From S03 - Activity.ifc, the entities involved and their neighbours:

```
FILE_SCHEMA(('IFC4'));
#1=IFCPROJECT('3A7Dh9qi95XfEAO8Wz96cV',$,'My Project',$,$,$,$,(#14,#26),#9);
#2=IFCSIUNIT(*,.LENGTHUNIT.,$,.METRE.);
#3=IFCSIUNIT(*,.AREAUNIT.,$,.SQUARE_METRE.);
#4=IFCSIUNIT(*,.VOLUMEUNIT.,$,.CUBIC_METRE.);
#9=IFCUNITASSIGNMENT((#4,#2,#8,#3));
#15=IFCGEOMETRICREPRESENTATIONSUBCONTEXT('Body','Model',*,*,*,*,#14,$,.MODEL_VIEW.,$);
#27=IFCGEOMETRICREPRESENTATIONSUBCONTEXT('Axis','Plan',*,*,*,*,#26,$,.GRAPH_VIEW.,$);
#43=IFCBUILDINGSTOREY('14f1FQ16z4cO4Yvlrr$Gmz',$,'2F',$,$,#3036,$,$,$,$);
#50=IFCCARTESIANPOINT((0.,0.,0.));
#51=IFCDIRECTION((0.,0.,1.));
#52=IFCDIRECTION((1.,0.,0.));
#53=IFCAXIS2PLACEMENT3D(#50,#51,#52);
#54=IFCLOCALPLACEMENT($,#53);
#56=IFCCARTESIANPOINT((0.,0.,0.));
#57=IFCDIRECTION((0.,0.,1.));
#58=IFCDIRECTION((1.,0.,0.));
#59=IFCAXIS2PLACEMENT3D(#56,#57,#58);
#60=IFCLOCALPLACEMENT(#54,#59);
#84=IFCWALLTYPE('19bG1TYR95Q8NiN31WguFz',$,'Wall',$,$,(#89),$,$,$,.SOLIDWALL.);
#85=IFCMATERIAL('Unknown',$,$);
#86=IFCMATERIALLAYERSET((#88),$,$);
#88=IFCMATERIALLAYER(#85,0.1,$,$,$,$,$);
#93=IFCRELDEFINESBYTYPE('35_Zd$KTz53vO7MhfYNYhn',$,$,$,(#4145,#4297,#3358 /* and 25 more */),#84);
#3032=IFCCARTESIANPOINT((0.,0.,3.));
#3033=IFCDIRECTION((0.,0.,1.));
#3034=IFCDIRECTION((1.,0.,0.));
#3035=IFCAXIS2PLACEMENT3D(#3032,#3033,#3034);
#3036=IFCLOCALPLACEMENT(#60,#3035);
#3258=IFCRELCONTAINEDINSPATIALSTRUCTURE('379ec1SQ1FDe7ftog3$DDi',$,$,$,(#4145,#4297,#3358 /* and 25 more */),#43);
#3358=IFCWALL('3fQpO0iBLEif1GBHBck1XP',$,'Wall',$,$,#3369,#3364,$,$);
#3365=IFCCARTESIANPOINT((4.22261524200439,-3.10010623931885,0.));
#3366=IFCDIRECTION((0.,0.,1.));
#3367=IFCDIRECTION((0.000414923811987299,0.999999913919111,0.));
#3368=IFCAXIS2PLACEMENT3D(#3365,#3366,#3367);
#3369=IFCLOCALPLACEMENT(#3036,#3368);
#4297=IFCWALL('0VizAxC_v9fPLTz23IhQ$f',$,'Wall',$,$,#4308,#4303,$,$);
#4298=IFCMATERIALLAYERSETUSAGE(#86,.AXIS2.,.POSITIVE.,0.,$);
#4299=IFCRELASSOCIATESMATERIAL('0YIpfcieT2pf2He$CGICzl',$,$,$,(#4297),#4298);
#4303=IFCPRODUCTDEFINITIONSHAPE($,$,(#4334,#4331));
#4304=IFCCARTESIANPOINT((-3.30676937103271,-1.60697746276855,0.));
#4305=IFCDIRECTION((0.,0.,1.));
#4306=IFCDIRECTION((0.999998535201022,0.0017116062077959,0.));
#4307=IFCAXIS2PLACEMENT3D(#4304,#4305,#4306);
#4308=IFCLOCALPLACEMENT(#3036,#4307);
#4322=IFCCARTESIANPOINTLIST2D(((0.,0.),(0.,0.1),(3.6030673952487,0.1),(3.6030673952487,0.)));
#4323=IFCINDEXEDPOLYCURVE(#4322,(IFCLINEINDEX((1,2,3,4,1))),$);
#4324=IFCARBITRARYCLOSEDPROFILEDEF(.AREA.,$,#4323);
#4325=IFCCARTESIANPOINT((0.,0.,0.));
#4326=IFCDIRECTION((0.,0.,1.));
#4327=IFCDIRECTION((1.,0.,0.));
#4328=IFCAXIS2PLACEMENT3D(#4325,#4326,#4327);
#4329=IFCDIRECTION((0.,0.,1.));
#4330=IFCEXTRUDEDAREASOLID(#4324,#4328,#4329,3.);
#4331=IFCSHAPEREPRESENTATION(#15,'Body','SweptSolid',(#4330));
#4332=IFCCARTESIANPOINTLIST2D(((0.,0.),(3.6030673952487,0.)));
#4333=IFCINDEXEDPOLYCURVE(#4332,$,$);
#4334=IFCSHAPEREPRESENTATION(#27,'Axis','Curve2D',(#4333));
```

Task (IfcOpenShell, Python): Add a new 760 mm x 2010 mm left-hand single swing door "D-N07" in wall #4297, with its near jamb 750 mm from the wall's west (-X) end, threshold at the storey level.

```python
import numpy as np
import ifcopenshell
import ifcopenshell.api.feature
import ifcopenshell.api.geometry
import ifcopenshell.api.root
import ifcopenshell.api.spatial
import ifcopenshell.geom
import ifcopenshell.util.element
import ifcopenshell.util.placement
import ifcopenshell.util.representation
import ifcopenshell.util.shape
import ifcopenshell.util.unit

model = ifcopenshell.open("S03 - Activity.ifc")
unit_scale = ifcopenshell.util.unit.calculate_unit_scale(model)
settings = ifcopenshell.geom.settings()


def volume(element):
    """Net volume in cubic metres, openings subtracted."""
    shape = ifcopenshell.geom.create_shape(settings, element)
    return ifcopenshell.util.shape.get_volume(shape.geometry)


wall = model.by_id(4297)
storey = ifcopenshell.util.element.get_container(wall, ifc_class="IfcBuildingStorey")
context = ifcopenshell.util.representation.get_context(model, "Model", "Body", "MODEL_VIEW")
before = volume(wall)

width, height, from_end, sill = 0.76, 2.01, 0.75, 0.0  # metres

# The wall runs along its own X axis, and the end named is its -X end.
wall_shape = ifcopenshell.geom.create_shape(settings, wall)
x, y, z = ifcopenshell.util.shape.get_vertices(wall_shape.geometry).T
start = x.min() + from_end
face, thickness = float(y.min()), float(y.max() - y.min())
wall_matrix = ifcopenshell.util.placement.get_local_placement(wall.ObjectPlacement)
level = ifcopenshell.util.placement.get_local_placement(storey.ObjectPlacement)[2, 3]


def in_wall(x, y):
    """Placement at x, y metres in the wall's axes, at sill height."""
    matrix = wall_matrix.copy()
    matrix[:, 3] = wall_matrix @ np.array([x / unit_scale, y / unit_scale, 0.0, 1.0])
    matrix[2, 3] = level + sill / unit_scale
    return matrix


# Opening: a box that overshoots both wall faces by 50 mm.
opening = ifcopenshell.api.root.create_entity(model, ifc_class="IfcOpeningElement", predefined_type="OPENING")
box = ifcopenshell.api.geometry.add_wall_representation(
    model, context=context, length=width, height=height, thickness=thickness + 0.1
)
ifcopenshell.api.geometry.assign_representation(model, product=opening, representation=box)
ifcopenshell.api.geometry.edit_object_placement(model, product=opening, matrix=in_wall(start, face - 0.05), is_si=False)
ifcopenshell.api.feature.add_feature(model, feature=opening, element=wall)

door = ifcopenshell.api.root.create_entity(model, ifc_class="IfcDoor", name="D-N07", predefined_type="DOOR")
door.OverallWidth, door.OverallHeight = width / unit_scale, height / unit_scale
door.OperationType = "SINGLE_SWING_LEFT"
body = ifcopenshell.api.geometry.add_door_representation(
    model,
    context=context,
    overall_width=door.OverallWidth,
    overall_height=door.OverallHeight,
    operation_type="SINGLE_SWING_LEFT",
    lining_properties={"LiningDepth": thickness / unit_scale, "ThresholdDepth": thickness / unit_scale},
)
ifcopenshell.api.geometry.assign_representation(model, product=door, representation=body)
ifcopenshell.api.spatial.assign_container(model, products=[door], relating_structure=storey)
ifcopenshell.api.feature.add_filling(model, opening=opening, element=door)

# The lining spans the wall, so the door starts at the wall face.
ifcopenshell.api.geometry.edit_object_placement(model, product=door, matrix=in_wall(start, face), is_si=False)

after = volume(wall)

print(f"wall volume {before:.3f} -> {after:.3f} m3")

model.write("S03 - Activity_updated.ifc")
```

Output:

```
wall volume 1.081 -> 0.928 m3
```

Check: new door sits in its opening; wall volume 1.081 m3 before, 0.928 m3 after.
